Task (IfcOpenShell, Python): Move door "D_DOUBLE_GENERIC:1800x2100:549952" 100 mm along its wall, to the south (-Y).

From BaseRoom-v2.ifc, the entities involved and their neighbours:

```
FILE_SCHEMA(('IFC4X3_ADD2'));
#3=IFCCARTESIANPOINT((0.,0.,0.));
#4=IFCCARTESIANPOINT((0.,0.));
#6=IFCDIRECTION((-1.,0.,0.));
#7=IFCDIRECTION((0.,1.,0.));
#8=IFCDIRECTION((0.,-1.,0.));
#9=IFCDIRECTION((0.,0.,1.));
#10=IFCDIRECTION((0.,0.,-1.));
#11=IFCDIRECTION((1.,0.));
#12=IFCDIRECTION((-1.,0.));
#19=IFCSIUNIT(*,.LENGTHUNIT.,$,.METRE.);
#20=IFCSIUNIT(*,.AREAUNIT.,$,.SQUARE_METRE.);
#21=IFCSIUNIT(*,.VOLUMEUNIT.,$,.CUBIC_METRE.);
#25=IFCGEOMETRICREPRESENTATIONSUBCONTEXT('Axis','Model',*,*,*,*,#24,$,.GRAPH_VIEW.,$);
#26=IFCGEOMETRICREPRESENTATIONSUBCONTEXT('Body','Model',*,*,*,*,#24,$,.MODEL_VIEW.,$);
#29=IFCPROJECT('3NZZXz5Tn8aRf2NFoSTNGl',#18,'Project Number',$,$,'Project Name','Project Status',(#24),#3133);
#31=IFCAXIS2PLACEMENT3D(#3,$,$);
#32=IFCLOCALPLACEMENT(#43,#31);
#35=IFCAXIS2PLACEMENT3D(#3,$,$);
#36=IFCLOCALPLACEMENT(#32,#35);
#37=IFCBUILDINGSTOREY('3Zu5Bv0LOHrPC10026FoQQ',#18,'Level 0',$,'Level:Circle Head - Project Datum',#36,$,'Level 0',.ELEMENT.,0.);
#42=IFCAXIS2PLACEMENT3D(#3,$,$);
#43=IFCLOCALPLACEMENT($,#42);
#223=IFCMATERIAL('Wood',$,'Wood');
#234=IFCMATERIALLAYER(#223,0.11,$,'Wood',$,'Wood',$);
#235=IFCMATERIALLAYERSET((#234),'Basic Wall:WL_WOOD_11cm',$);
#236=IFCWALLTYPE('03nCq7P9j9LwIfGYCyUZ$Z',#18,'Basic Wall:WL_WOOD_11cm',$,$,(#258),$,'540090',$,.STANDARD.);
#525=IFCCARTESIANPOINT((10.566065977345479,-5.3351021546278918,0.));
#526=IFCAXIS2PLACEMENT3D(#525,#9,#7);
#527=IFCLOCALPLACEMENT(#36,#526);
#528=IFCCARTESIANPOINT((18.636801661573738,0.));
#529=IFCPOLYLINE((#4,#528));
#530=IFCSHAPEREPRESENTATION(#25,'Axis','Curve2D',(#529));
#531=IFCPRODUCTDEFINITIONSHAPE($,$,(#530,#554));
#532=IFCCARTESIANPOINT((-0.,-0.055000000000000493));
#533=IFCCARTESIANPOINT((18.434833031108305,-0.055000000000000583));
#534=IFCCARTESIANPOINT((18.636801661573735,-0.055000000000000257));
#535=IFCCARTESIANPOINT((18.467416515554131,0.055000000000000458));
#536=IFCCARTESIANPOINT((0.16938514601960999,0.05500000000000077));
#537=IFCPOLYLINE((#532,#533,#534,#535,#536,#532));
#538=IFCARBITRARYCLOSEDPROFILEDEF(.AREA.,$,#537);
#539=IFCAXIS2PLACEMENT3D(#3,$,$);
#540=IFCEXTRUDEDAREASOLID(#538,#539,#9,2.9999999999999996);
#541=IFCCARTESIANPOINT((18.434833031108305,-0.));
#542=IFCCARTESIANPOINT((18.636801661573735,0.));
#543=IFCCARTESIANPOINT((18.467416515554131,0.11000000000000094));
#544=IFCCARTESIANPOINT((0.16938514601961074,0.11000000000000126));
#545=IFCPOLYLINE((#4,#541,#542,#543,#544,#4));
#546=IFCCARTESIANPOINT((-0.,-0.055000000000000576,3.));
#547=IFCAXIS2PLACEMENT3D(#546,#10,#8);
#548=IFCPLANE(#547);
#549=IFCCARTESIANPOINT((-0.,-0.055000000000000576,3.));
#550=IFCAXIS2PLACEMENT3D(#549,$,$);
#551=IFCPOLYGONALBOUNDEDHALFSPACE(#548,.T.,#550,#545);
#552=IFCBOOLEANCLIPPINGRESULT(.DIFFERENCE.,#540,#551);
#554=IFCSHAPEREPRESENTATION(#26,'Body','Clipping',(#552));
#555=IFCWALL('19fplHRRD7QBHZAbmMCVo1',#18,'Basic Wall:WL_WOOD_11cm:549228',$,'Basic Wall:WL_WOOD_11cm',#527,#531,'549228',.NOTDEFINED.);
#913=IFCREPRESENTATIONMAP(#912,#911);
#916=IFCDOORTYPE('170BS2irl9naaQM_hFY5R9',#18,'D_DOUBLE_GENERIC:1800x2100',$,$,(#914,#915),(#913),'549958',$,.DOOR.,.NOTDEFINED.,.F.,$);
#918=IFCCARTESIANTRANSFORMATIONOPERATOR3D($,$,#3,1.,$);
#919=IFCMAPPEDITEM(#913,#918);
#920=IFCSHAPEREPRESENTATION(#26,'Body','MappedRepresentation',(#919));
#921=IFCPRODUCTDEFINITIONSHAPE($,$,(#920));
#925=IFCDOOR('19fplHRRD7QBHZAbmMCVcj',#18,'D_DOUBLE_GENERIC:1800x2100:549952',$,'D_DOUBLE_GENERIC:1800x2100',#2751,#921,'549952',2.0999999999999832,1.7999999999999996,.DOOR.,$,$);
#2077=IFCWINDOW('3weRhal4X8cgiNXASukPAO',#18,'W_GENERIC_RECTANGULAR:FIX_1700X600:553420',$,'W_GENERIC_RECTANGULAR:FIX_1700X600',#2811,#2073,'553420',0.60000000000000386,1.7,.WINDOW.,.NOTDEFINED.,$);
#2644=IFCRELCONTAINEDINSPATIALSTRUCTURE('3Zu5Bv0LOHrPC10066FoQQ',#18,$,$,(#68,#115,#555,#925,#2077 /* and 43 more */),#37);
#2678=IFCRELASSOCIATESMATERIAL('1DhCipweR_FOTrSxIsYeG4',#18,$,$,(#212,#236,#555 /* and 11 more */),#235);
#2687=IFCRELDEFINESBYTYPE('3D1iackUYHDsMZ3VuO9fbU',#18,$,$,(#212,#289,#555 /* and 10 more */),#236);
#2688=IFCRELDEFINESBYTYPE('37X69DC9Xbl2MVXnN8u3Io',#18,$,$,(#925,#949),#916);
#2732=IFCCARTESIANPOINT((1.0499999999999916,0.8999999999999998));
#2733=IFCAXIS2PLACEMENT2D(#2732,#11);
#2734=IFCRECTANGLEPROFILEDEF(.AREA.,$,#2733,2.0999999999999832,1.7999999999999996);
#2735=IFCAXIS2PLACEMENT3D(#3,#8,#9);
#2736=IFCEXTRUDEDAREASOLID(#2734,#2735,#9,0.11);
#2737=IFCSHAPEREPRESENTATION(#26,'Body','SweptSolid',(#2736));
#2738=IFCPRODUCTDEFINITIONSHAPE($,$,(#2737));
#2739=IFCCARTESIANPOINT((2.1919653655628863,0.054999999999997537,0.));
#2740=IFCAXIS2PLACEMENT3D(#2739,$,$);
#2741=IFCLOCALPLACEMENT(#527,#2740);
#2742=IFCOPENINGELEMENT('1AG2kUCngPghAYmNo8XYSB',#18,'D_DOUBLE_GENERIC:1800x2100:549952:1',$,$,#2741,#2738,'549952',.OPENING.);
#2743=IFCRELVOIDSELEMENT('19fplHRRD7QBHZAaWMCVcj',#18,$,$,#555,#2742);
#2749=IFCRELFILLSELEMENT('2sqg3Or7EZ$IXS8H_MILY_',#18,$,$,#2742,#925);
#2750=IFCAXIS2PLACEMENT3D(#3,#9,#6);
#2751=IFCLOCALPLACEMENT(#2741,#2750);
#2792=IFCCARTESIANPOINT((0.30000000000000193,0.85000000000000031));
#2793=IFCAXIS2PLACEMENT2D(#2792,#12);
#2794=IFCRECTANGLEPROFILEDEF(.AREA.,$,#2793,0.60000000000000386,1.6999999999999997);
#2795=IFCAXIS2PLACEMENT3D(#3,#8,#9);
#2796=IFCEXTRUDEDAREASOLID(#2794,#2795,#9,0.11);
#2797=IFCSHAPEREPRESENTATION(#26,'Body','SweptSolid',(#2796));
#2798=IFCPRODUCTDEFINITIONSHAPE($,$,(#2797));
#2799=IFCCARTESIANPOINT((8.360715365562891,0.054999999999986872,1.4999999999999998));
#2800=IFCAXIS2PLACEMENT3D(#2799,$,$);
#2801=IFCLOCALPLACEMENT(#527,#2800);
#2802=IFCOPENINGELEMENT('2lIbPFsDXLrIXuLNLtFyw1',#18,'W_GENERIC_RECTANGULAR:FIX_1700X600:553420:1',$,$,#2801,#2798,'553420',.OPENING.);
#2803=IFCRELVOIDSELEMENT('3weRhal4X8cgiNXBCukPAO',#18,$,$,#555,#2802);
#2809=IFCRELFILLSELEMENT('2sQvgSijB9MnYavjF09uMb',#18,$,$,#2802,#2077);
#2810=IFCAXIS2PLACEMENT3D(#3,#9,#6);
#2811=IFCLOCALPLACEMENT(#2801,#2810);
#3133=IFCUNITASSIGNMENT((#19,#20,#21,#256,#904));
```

```python
import ifcopenshell
import ifcopenshell.api.geometry
import ifcopenshell.util.placement

model = ifcopenshell.open("BaseRoom-v2.ifc")

door = model.by_guid("19fplHRRD7QBHZAbmMCVcj")
opening = door.FillsVoids[0].RelatingOpeningElement
wall = opening.VoidsElements[0].RelatingBuildingElement

wall_matrix = ifcopenshell.util.placement.get_local_placement(wall.ObjectPlacement)
shift = wall_matrix[:3, 0] * -0.1
before = ifcopenshell.util.placement.get_local_placement(door.ObjectPlacement)[:3, 3].copy()

# The door is placed relative to its opening, so it follows when the opening moves.
matrix = ifcopenshell.util.placement.get_local_placement(opening.ObjectPlacement)
matrix[:3, 3] += shift
ifcopenshell.api.geometry.edit_object_placement(
    model, product=opening, matrix=matrix, is_si=False, should_transform_children=True
)

after = ifcopenshell.util.placement.get_local_placement(door.ObjectPlacement)[:3, 3]
print("door moved by", (after - before).round(3) + 0.0)

model.write("BaseRoom-v2-out.ifc")
```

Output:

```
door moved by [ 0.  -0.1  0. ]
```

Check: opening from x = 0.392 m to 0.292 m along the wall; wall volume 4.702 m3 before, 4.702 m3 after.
